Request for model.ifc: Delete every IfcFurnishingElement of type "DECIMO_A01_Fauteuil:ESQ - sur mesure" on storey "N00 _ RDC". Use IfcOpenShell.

First a look at what the model holds.

```python
import ifcopenshell
import ifcopenshell.util.element

model = ifcopenshell.open("model.ifc")
print(model.schema)
storey = next(s for s in model.by_type("IfcBuildingStorey") if s.Name == "N00 _ RDC")
furniture = [e for e in ifcopenshell.util.element.get_decomposition(storey) if e.is_a("IfcFurnishingElement")]
seen = {}
for e in furniture:
    element_type = ifcopenshell.util.element.get_type(e)
    name = element_type.Name if element_type not in (None, e) else None
    seen[name] = seen.get(name, 0) + 1
for name, count in sorted(seen.items(), key=str):
    print(count, "x", name)
```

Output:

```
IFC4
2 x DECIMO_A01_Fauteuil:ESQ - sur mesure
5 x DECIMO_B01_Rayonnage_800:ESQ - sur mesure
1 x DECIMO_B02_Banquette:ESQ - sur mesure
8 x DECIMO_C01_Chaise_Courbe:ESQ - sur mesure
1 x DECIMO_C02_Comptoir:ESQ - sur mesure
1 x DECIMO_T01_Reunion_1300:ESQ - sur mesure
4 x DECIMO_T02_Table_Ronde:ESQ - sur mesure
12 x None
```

```python
import ifcopenshell
import ifcopenshell.api.root
import ifcopenshell.util.element

model = ifcopenshell.open("model.ifc")

storey = next(s for s in model.by_type("IfcBuildingStorey") if s.Name == "N00 _ RDC")
furniture = [e for e in ifcopenshell.util.element.get_decomposition(storey) if e.is_a("IfcFurnishingElement")]
targets = [e for e in furniture if (t := ifcopenshell.util.element.get_type(e)) not in (None, e) and t.Name == "DECIMO_A01_Fauteuil:ESQ - sur mesure"]

for e in targets:
    ifcopenshell.api.root.remove_product(model, product=e)
print(len(targets), "removed")

model.write("model_edited.ifc")
```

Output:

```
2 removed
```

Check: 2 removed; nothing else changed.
